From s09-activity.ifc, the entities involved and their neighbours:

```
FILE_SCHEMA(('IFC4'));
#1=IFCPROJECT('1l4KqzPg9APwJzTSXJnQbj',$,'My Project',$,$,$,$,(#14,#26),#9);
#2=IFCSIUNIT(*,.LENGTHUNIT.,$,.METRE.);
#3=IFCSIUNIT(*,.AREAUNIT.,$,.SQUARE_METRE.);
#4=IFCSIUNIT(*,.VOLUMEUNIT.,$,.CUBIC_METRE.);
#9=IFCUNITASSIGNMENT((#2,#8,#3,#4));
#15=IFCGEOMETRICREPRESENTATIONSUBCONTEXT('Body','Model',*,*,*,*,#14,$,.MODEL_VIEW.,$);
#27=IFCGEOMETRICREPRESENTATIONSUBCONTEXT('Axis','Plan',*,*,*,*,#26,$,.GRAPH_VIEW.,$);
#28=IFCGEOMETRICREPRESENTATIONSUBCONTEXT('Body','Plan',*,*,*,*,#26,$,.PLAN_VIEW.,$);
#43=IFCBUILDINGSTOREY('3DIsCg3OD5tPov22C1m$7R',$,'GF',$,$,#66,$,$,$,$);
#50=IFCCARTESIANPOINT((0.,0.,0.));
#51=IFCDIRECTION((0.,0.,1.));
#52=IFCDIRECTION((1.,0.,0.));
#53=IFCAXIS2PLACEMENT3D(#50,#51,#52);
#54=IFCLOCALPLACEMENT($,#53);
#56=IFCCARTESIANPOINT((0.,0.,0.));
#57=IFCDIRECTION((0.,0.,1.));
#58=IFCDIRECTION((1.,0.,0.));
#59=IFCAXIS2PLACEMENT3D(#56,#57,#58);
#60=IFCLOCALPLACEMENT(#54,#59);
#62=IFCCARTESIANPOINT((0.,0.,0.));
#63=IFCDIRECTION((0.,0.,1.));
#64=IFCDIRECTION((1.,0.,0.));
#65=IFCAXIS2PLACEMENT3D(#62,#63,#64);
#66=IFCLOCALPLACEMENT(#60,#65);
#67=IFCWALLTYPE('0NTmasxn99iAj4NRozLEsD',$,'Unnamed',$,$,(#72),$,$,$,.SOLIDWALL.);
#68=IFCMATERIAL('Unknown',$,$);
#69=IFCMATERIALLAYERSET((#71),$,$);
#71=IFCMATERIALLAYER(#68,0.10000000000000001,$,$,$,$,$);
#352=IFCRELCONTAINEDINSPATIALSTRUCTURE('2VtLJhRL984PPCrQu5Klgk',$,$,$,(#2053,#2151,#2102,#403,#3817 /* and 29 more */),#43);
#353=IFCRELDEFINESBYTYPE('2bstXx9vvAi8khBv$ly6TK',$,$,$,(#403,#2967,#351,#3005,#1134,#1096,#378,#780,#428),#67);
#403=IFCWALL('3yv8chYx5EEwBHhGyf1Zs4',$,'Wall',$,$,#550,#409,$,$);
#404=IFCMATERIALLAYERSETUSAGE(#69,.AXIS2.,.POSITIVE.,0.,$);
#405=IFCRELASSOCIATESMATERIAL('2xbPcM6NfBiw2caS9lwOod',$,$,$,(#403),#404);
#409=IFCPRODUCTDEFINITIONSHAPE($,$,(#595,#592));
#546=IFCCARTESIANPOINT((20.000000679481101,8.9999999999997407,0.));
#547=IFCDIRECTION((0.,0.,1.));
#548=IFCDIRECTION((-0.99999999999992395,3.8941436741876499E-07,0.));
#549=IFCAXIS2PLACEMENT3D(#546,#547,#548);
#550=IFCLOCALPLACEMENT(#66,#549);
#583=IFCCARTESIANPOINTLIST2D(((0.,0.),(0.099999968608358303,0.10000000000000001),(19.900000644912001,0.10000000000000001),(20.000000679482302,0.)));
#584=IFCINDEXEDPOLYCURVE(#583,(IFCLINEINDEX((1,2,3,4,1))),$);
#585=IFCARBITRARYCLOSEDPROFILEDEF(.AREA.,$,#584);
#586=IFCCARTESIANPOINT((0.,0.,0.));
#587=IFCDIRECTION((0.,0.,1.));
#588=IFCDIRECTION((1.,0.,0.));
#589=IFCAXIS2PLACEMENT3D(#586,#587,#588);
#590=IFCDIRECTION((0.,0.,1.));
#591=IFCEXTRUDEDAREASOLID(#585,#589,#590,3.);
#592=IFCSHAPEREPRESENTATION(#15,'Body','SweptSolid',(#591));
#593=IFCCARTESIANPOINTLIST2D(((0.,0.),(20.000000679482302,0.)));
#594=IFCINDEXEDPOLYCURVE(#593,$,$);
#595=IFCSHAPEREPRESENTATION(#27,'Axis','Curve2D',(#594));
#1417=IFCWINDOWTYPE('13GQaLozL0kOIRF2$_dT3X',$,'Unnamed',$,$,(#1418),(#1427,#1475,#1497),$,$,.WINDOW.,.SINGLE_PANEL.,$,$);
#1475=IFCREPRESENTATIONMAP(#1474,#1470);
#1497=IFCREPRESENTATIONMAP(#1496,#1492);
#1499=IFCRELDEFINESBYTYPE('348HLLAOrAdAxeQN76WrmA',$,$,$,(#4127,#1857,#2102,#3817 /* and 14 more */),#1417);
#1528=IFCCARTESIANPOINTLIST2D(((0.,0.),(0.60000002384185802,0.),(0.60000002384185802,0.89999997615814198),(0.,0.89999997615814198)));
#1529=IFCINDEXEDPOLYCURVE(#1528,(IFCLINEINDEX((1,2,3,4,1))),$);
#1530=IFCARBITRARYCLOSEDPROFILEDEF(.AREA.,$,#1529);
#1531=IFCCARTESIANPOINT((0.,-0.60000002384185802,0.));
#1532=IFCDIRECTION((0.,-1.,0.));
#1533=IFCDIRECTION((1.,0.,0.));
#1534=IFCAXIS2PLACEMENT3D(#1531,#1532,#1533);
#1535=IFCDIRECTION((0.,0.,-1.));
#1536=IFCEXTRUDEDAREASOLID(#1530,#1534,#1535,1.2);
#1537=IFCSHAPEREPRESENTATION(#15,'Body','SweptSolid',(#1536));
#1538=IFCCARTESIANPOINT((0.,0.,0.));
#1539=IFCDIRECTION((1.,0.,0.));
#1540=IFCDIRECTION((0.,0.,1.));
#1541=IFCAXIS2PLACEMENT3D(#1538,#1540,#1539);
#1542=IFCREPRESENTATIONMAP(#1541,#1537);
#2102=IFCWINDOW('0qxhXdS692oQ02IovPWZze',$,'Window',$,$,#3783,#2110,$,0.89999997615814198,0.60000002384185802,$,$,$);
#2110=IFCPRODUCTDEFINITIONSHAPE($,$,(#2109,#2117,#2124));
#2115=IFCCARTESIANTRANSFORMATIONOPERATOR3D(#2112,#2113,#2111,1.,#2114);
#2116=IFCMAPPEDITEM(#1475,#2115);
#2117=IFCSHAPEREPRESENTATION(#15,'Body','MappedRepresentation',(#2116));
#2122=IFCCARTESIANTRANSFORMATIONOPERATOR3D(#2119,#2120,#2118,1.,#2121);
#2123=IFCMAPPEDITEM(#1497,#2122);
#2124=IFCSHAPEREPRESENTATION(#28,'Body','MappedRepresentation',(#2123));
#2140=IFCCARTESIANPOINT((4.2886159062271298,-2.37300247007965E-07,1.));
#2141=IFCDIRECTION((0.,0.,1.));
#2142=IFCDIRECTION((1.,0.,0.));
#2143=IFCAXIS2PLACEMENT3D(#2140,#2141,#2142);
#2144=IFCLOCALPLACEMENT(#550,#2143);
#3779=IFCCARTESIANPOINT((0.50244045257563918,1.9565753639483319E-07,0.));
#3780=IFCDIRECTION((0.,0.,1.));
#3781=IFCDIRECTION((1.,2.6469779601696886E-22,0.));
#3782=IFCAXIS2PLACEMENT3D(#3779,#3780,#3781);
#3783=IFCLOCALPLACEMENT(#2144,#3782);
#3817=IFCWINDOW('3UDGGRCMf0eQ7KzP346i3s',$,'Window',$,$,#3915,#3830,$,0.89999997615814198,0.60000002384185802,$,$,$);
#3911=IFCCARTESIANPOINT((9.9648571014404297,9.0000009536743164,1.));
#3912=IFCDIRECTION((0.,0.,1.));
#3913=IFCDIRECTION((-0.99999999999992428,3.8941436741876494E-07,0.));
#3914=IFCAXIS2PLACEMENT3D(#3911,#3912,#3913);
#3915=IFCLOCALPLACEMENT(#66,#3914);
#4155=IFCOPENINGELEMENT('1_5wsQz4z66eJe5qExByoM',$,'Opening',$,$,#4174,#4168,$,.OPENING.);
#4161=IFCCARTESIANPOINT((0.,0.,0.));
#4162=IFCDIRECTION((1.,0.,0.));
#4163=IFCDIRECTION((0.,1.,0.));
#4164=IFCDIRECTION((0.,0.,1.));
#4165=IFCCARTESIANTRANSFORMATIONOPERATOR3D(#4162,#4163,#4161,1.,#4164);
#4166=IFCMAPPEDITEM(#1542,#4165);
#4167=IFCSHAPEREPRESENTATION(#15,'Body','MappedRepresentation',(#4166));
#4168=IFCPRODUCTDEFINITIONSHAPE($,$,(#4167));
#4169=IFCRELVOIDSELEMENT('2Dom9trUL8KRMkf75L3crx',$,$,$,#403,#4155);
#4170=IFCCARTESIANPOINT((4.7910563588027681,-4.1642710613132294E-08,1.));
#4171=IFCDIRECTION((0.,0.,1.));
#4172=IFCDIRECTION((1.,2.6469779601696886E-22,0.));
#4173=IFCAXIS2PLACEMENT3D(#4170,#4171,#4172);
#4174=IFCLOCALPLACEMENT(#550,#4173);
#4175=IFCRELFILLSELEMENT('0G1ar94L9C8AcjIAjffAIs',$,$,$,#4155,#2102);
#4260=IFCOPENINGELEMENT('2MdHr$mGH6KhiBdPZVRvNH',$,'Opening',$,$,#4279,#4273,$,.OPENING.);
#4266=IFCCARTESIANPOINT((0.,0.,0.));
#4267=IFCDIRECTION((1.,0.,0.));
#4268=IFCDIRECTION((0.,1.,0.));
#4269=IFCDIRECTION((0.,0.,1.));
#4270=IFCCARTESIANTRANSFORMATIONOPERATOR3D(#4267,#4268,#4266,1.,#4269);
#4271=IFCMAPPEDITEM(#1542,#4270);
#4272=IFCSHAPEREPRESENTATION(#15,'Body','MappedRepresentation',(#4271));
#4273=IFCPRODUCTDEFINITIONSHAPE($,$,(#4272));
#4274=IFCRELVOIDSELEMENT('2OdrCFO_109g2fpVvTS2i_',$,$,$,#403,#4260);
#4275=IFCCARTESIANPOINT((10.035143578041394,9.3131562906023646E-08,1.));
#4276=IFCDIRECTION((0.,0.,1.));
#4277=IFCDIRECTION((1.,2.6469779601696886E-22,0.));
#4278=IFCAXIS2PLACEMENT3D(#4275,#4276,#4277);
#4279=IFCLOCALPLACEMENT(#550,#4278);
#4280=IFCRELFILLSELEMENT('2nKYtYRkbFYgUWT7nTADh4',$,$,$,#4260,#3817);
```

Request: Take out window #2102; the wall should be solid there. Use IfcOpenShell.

```python
import ifcopenshell
import ifcopenshell.api.feature
import ifcopenshell.api.root
import ifcopenshell.geom
import ifcopenshell.util.shape

model = ifcopenshell.open("s09-activity.ifc")
settings = ifcopenshell.geom.settings()


def volume(element):
    """Net volume in cubic metres, openings subtracted."""
    shape = ifcopenshell.geom.create_shape(settings, element)
    return ifcopenshell.util.shape.get_volume(shape.geometry)


window = model.by_guid("0qxhXdS692oQ02IovPWZze")
opening = window.FillsVoids[0].RelatingOpeningElement
wall = opening.VoidsElements[0].RelatingBuildingElement
before = volume(wall)

ifcopenshell.api.root.remove_product(model, product=window)
ifcopenshell.api.feature.remove_feature(model, feature=opening)

after = volume(wall)

print(f"wall volume {before:.3f} -> {after:.3f} m3")

model.write("s09-activity_updated.ifc")
```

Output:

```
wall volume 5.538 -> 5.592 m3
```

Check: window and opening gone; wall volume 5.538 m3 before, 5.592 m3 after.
